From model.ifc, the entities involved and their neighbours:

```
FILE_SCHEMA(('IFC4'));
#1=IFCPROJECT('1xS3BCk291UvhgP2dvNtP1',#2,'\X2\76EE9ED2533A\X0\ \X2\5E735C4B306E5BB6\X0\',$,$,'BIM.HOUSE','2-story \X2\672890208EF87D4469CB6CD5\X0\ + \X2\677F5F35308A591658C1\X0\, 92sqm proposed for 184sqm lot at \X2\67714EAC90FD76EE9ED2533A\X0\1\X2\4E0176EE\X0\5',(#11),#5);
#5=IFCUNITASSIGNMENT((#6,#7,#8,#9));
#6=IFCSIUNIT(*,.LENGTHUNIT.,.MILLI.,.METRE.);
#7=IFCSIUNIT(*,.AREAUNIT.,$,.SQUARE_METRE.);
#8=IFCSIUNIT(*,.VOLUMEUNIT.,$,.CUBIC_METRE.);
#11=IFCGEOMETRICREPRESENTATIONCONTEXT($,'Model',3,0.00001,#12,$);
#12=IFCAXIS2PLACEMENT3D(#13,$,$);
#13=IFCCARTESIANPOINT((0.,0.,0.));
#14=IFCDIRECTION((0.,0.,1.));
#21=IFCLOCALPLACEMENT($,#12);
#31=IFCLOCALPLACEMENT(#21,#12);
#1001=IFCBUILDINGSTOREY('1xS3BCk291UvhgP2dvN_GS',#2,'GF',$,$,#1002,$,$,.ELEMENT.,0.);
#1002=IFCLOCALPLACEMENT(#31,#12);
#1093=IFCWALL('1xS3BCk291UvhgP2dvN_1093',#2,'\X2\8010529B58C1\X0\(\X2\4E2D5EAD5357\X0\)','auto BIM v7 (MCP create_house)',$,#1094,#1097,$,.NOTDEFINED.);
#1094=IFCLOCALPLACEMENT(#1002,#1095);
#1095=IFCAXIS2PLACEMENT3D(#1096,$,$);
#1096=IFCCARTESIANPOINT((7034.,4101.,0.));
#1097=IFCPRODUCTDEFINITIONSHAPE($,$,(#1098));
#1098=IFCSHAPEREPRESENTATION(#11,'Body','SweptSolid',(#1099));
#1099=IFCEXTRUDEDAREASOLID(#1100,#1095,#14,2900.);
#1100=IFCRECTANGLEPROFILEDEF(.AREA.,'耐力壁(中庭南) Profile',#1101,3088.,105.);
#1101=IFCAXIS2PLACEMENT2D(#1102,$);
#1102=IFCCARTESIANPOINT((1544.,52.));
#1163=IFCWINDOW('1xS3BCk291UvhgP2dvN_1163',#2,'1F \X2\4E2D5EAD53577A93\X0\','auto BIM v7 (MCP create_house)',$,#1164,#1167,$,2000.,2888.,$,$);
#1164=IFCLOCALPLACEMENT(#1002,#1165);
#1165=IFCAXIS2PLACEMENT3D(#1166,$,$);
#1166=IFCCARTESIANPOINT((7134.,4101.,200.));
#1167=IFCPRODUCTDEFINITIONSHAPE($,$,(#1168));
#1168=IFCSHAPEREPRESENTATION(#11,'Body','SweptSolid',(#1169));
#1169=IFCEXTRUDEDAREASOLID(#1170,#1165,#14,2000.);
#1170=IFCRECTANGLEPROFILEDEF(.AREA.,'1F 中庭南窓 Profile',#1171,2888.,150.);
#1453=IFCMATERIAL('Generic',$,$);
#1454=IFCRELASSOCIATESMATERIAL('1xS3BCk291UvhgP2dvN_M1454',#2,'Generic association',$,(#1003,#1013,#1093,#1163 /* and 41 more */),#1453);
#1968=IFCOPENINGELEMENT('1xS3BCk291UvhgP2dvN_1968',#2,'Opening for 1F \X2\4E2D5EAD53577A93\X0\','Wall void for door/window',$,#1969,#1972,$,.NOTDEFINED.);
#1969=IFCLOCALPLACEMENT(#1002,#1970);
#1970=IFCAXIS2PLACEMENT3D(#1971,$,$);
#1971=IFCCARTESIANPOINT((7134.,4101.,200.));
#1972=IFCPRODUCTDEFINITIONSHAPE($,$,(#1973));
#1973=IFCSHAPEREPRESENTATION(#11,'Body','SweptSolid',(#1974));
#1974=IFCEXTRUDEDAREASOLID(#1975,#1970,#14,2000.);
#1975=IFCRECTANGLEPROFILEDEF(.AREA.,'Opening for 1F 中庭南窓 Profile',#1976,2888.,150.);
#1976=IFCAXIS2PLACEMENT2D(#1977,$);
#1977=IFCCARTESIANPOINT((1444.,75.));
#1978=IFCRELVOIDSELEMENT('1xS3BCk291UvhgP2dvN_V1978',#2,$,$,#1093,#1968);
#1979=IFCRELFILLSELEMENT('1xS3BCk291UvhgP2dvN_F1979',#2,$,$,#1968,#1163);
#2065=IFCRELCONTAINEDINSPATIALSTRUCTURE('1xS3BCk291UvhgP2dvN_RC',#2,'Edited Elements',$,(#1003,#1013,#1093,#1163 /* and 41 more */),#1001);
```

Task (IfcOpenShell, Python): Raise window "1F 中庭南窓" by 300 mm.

```python
import numpy as np
import ifcopenshell
import ifcopenshell.api.geometry
import ifcopenshell.util.placement
import ifcopenshell.util.unit

model = ifcopenshell.open("model.ifc")
unit_scale = ifcopenshell.util.unit.calculate_unit_scale(model)

window = model.by_id(1163)
opening = window.FillsVoids[0].RelatingOpeningElement
dz = 0.3 / unit_scale

shift = np.array([0.0, 0.0, dz])
# The window is not placed relative to its opening, so move both.
for product in (opening, window):
    matrix = ifcopenshell.util.placement.get_local_placement(product.ObjectPlacement)
    matrix[:3, 3] += shift
    ifcopenshell.api.geometry.edit_object_placement(model, product=product, matrix=matrix, is_si=False)

print(f"moved by {dz * unit_scale:+.3f} m")

model.write("model_edited.ifc")
```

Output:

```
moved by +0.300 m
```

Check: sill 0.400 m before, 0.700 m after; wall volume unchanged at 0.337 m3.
